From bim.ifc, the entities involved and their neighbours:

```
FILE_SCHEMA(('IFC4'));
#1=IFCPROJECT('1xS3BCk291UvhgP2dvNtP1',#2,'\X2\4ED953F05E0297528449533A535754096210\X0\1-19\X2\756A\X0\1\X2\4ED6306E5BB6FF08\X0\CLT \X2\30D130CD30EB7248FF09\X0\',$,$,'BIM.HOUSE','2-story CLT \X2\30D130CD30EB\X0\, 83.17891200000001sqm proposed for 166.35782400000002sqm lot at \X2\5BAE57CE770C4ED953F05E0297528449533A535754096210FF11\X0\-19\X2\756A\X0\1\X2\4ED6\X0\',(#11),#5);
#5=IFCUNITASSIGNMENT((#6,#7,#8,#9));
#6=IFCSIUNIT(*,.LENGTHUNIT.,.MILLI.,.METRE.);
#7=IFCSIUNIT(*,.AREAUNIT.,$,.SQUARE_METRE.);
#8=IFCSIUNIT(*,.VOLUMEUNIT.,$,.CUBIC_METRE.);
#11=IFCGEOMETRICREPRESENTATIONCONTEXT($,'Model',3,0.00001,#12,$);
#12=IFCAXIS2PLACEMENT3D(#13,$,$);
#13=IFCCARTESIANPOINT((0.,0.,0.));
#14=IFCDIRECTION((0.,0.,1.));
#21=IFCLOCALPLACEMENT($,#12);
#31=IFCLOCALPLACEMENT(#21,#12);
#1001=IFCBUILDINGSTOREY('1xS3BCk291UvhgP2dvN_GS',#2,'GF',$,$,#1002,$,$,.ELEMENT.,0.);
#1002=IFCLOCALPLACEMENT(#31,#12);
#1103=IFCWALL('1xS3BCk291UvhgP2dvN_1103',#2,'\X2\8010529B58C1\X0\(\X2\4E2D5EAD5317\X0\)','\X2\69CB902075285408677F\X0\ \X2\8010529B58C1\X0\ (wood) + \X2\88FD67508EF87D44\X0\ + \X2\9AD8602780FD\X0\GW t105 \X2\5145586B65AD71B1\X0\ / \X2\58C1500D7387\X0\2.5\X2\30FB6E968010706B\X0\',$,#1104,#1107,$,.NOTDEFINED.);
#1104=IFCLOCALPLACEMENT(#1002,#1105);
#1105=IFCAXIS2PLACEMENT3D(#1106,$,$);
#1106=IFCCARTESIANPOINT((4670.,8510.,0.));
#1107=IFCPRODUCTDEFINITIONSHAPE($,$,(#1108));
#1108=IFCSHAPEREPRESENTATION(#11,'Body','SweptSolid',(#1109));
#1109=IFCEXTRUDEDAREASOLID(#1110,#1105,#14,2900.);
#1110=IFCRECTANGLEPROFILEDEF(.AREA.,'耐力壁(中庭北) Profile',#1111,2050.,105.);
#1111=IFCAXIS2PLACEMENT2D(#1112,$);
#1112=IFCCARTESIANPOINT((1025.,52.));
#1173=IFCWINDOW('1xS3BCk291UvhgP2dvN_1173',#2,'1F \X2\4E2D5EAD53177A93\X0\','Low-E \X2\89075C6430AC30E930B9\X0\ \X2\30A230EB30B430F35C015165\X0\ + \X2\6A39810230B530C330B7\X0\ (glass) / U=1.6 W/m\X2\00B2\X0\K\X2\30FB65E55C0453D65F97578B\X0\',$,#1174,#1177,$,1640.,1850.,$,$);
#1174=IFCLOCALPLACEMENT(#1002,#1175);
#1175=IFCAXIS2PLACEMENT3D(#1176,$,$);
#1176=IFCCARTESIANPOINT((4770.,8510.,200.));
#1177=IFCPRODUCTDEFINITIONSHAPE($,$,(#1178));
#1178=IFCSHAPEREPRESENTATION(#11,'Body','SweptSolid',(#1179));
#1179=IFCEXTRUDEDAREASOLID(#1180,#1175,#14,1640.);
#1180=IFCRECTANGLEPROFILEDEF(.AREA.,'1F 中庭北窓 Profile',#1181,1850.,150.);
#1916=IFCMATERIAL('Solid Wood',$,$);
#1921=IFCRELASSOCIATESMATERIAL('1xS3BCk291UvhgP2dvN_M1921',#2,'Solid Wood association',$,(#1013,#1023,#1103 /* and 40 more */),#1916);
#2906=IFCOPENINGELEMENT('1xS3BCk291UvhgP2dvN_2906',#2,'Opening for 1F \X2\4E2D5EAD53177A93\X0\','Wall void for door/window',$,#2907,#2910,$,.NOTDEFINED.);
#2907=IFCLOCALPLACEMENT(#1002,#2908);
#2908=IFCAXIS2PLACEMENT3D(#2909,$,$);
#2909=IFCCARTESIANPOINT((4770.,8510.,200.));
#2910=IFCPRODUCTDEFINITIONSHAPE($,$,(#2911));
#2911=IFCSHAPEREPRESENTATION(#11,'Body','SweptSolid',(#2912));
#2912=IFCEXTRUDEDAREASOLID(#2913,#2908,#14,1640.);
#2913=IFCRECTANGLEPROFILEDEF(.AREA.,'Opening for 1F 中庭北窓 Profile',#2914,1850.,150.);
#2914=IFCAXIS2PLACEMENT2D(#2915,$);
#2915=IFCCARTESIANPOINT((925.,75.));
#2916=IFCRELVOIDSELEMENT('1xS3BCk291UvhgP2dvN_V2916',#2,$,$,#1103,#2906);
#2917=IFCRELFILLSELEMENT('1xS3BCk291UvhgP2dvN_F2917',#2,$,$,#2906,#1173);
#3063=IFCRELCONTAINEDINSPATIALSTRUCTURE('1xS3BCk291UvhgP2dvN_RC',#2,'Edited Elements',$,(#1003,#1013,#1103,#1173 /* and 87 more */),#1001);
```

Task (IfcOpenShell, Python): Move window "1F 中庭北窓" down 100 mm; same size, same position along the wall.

```python
import numpy as np
import ifcopenshell
import ifcopenshell.api.geometry
import ifcopenshell.util.placement
import ifcopenshell.util.unit

model = ifcopenshell.open("bim.ifc")
unit_scale = ifcopenshell.util.unit.calculate_unit_scale(model)

window = model.by_guid("1xS3BCk291UvhgP2dvN_1173")
opening = window.FillsVoids[0].RelatingOpeningElement
dz = -100.0

shift = np.array([0.0, 0.0, dz])
# The window is not placed relative to its opening, so move both.
for product in (opening, window):
    matrix = ifcopenshell.util.placement.get_local_placement(product.ObjectPlacement)
    matrix[:3, 3] += shift
    ifcopenshell.api.geometry.edit_object_placement(model, product=product, matrix=matrix, is_si=False)

print(f"moved by {dz * unit_scale:+.3f} m")

model.write("bim_edited.ifc")
```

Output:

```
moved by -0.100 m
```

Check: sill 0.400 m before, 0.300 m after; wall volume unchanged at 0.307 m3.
